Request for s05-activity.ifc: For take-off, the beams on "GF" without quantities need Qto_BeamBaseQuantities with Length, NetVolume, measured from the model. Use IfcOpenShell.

First a look at what the model holds.

```python
import ifcopenshell
import ifcopenshell.util.element
import ifcopenshell.util.unit

model = ifcopenshell.open("s05-activity.ifc")
print(model.schema)
for unit_type in ("LENGTHUNIT", "AREAUNIT", "VOLUMEUNIT"):
    print(unit_type, ifcopenshell.util.unit.calculate_unit_scale(model, unit_type))
storey = next(s for s in model.by_type("IfcBuildingStorey") if s.Name == "GF")
beams = [e for e in ifcopenshell.util.element.get_decomposition(storey) if e.is_a("IfcBeam")]
for e in sorted(beams, key=lambda e: e.id()):
    print(e.id(), e.is_a(), e.Name, list(ifcopenshell.util.element.get_psets(e, qtos_only=True)), sep=" | ")
```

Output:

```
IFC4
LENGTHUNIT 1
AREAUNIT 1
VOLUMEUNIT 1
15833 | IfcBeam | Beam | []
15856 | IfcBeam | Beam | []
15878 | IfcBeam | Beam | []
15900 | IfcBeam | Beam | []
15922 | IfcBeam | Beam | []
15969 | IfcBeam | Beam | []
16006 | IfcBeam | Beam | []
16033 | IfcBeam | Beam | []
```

```python
import ifcopenshell
import ifcopenshell.api.pset
import ifcopenshell.geom
import ifcopenshell.util.element
import ifcopenshell.util.shape
import ifcopenshell.util.unit

model = ifcopenshell.open("s05-activity.ifc")
unit_scale = ifcopenshell.util.unit.calculate_unit_scale(model)
volume_scale = ifcopenshell.util.unit.calculate_unit_scale(model, "VOLUMEUNIT")
settings = ifcopenshell.geom.settings()

storey = next(s for s in model.by_type("IfcBuildingStorey") if s.Name == "GF")
beams = [e for e in ifcopenshell.util.element.get_decomposition(storey) if e.is_a("IfcBeam")]

for e in sorted(beams, key=lambda e: e.id()):
    if ifcopenshell.util.element.get_psets(e, qtos_only=True, should_inherit=False):
        continue
    # Geometry comes back in metres, in the element's own axes.
    shape = ifcopenshell.geom.create_shape(settings, e)
    values = {
        "Length": ifcopenshell.util.shape.get_max_xyz(shape.geometry) / unit_scale,
        "NetVolume": ifcopenshell.util.shape.get_volume(shape.geometry) / volume_scale,
    }
    qto = ifcopenshell.api.pset.add_qto(model, product=e, name="Qto_BeamBaseQuantities")
    ifcopenshell.api.pset.edit_qto(model, qto=qto, properties=values)
    print(e.id(), {k: round(v, 3) for k, v in values.items()})

model.write("s05-activity_rev.ifc")
```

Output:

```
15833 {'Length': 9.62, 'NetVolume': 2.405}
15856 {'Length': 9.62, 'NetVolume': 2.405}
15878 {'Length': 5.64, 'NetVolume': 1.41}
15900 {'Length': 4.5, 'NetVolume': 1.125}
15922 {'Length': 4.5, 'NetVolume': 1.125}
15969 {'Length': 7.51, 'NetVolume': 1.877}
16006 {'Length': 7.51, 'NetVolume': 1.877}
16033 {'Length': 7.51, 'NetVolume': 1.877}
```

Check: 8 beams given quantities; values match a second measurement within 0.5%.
